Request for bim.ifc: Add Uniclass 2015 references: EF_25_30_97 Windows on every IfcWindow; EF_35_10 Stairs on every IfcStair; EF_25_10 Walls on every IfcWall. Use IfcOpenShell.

First a look at what the model holds.

```python
import ifcopenshell

model = ifcopenshell.open("bim.ifc")
print(model.schema)
print("classifications:", [c.Name for c in model.by_type("IfcClassification")])
for ifc_class in ("IfcDoor", "IfcRoof", "IfcStair", "IfcWall", "IfcWindow"):
    print(ifc_class, len(model.by_type(ifc_class)))
```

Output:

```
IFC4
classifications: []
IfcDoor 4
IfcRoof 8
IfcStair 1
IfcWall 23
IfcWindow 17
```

```python
import ifcopenshell
import ifcopenshell.api.classification

model = ifcopenshell.open("bim.ifc")

system = ifcopenshell.api.classification.add_classification(model, classification="Uniclass 2015")

codes = {
    "IfcWindow": ("EF_25_30_97", "Windows"),
    "IfcStair": ("EF_35_10", "Stairs"),
    "IfcWall": ("EF_25_10", "Walls"),
}
for ifc_class, (code, name) in codes.items():
    products = model.by_type(ifc_class)
    ifcopenshell.api.classification.add_reference(
        model, products=products, classification=system, identification=code, name=name
    )
    print(code, len(products))

model.write("bim_updated.ifc")
```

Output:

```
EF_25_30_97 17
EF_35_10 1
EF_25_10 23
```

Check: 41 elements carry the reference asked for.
